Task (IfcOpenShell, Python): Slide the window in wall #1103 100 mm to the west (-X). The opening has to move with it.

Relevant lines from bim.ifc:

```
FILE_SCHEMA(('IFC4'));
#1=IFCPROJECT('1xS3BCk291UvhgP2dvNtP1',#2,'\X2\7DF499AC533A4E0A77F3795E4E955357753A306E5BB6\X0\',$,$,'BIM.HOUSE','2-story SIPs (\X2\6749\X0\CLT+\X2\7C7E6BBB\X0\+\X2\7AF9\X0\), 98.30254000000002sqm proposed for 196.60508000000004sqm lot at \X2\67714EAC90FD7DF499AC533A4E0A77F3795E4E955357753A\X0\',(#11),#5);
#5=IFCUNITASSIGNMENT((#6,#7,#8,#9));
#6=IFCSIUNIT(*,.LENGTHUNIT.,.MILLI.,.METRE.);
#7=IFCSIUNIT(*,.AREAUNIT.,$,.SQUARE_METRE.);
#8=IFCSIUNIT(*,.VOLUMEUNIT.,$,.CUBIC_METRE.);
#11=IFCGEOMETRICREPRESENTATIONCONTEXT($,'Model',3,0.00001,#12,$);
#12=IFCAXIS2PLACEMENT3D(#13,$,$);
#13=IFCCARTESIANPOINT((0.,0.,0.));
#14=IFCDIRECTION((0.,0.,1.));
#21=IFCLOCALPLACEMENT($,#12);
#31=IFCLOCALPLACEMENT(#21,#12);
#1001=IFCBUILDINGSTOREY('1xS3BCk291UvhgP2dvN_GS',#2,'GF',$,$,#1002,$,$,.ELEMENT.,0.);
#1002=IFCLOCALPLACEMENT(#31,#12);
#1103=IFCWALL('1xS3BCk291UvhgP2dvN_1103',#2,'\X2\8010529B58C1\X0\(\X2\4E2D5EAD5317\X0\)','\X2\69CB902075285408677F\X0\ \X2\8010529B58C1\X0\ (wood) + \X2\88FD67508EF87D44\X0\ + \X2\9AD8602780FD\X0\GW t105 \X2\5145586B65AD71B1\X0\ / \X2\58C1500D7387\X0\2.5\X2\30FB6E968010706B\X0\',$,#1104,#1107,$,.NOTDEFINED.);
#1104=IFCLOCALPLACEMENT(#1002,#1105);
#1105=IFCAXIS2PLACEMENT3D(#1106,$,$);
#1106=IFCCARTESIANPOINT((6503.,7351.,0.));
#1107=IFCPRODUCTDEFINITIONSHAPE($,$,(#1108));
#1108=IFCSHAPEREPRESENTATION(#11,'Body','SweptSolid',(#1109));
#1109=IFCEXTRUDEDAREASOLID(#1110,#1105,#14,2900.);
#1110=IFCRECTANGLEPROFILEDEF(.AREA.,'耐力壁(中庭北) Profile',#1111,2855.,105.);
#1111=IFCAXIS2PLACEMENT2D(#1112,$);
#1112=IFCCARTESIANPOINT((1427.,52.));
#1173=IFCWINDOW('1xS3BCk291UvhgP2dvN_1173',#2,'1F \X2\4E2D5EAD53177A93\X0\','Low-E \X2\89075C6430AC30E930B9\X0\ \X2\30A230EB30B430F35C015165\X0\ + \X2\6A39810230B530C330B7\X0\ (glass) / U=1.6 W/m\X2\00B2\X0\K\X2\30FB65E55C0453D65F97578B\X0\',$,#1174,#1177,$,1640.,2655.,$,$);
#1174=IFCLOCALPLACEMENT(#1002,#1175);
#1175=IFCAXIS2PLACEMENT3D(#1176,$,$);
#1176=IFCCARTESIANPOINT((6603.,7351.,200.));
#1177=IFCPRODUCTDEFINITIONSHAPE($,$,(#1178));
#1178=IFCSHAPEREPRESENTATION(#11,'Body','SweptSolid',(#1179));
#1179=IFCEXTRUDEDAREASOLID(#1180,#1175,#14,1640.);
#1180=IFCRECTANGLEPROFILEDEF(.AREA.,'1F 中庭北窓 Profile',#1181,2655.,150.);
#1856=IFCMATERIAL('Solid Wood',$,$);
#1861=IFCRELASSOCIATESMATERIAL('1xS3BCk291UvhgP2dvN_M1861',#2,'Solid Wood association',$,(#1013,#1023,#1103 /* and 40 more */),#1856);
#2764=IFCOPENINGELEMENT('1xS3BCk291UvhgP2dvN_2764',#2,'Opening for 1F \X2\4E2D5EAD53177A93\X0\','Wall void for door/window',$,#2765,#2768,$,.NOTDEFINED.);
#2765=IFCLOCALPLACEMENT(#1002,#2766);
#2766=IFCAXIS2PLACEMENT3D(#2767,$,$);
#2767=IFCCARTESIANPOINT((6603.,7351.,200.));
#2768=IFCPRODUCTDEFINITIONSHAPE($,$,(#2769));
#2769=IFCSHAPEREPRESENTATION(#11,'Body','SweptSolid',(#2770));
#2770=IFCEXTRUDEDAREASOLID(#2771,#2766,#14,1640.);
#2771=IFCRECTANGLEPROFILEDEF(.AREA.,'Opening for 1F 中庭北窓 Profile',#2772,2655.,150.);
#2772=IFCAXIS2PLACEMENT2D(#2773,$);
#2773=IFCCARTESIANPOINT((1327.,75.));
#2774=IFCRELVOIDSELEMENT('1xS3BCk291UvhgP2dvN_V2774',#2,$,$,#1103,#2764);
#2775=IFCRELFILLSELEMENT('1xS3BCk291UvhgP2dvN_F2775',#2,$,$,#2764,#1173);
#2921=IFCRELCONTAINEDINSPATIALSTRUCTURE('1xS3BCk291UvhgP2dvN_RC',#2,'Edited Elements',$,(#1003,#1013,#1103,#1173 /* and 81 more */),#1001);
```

```python
import ifcopenshell
import ifcopenshell.api.geometry
import ifcopenshell.util.placement
import ifcopenshell.util.unit

model = ifcopenshell.open("bim.ifc")
unit_scale = ifcopenshell.util.unit.calculate_unit_scale(model)

window = model.by_id(1173)
opening = window.FillsVoids[0].RelatingOpeningElement
wall = opening.VoidsElements[0].RelatingBuildingElement

wall_matrix = ifcopenshell.util.placement.get_local_placement(wall.ObjectPlacement)
shift = wall_matrix[:3, 0] * -0.1 / unit_scale
before = ifcopenshell.util.placement.get_local_placement(window.ObjectPlacement)[:3, 3].copy()

# The window is not placed relative to its opening, so move both.
for product in (opening, window):
    matrix = ifcopenshell.util.placement.get_local_placement(product.ObjectPlacement)
    matrix[:3, 3] += shift
    ifcopenshell.api.geometry.edit_object_placement(model, product=product, matrix=matrix, is_si=False)

after = ifcopenshell.util.placement.get_local_placement(window.ObjectPlacement)[:3, 3]
print("window moved by", (after - before).round(3) + 0.0)

model.write("bim_updated.ifc")
```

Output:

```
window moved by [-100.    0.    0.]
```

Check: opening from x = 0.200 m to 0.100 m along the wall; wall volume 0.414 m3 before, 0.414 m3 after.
